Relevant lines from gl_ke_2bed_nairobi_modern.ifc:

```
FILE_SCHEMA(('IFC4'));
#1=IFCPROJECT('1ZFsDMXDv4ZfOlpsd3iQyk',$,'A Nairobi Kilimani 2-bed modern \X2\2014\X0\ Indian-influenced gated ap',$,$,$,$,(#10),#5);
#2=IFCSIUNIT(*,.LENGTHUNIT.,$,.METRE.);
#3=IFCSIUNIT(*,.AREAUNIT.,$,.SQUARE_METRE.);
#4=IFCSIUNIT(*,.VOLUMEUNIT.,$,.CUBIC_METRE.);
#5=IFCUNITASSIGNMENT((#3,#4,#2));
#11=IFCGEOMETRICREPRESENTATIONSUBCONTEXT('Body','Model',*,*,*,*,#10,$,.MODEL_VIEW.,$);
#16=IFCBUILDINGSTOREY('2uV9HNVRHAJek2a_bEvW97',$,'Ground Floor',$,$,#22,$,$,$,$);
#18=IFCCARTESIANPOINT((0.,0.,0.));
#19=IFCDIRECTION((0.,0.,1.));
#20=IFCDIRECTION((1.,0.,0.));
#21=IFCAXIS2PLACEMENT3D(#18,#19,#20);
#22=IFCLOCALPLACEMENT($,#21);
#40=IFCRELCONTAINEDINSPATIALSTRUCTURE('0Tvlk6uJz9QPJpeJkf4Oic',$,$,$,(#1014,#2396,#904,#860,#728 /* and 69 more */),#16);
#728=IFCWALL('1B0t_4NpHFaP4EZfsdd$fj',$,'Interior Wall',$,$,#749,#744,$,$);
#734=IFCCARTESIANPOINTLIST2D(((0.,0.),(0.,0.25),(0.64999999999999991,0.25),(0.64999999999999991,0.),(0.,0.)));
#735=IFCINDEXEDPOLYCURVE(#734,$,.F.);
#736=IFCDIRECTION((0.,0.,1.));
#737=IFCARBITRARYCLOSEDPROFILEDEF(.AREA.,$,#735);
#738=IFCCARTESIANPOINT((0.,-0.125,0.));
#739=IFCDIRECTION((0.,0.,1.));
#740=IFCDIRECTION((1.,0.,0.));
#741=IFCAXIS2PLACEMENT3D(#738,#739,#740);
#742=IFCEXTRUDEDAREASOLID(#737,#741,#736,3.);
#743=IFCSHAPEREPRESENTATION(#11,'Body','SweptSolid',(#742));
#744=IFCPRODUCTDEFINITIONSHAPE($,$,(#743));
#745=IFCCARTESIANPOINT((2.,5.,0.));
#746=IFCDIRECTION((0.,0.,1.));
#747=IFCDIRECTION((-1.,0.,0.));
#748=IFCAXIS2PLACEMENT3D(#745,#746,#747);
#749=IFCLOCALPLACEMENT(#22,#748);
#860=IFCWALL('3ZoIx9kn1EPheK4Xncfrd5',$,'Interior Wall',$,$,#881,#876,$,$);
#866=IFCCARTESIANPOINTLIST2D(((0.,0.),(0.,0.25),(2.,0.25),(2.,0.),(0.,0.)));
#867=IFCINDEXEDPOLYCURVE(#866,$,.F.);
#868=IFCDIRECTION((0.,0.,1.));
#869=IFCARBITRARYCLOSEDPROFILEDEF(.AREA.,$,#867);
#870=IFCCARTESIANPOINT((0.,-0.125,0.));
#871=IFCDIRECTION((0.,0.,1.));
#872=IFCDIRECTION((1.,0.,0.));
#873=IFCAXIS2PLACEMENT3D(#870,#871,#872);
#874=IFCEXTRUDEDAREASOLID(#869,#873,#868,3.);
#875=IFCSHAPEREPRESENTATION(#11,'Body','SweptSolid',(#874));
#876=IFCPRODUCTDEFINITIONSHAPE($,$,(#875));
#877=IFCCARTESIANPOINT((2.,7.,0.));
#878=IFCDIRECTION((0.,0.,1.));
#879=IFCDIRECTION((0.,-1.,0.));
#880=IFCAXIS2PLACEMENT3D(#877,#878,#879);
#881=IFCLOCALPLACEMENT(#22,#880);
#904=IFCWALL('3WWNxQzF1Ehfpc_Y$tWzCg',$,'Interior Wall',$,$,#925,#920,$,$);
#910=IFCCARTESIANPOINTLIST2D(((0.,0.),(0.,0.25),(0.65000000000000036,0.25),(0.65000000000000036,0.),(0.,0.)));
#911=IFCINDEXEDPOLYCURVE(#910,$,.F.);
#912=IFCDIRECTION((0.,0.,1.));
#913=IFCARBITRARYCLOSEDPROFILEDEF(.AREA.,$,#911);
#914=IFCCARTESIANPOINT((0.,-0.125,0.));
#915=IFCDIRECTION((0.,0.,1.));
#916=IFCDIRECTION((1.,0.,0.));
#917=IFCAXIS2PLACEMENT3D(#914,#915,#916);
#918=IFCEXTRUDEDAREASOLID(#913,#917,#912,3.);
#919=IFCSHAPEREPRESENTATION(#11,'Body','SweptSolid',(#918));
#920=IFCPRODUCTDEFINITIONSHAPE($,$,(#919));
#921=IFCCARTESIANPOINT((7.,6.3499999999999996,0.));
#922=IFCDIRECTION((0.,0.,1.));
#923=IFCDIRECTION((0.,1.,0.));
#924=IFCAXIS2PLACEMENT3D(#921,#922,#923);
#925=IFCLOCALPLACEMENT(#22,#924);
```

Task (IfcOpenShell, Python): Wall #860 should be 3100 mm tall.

```python
import ifcopenshell
import ifcopenshell.geom
import ifcopenshell.util.representation
import ifcopenshell.util.shape
import ifcopenshell.util.unit

model = ifcopenshell.open("gl_ke_2bed_nairobi_modern.ifc")
unit_scale = ifcopenshell.util.unit.calculate_unit_scale(model)
settings = ifcopenshell.geom.settings()


def volume(element):
    """Net volume in cubic metres, openings subtracted."""
    shape = ifcopenshell.geom.create_shape(settings, element)
    return ifcopenshell.util.shape.get_volume(shape.geometry)


wall = model.by_guid("3ZoIx9kn1EPheK4Xncfrd5")
before = volume(wall)

body = ifcopenshell.util.representation.get_representation(wall, "Model", "Body")
solid = body.Items[0]
old_height = solid.Depth
solid.Depth = 3.1 / unit_scale
after = volume(wall)

print(f"height {old_height:g} -> {solid.Depth:g}, volume {before:.3f} -> {after:.3f} m3")

model.write("gl_ke_2bed_nairobi_modern_updated.ifc")
```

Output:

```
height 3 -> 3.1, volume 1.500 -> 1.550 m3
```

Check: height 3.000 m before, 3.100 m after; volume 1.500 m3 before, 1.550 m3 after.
